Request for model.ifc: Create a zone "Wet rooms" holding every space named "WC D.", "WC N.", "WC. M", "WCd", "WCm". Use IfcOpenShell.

First a look at what the model holds.

```python
import ifcopenshell

model = ifcopenshell.open("model.ifc")
print(model.schema)
seen = {}
for space in model.by_type("IfcSpace"):
    seen[space.LongName] = seen.get(space.LongName, 0) + 1
for name, count in sorted(seen.items(), key=str):
    print(count, "x", name)
print("zones:", [z.Name for z in model.by_type("IfcZone")][:20])
```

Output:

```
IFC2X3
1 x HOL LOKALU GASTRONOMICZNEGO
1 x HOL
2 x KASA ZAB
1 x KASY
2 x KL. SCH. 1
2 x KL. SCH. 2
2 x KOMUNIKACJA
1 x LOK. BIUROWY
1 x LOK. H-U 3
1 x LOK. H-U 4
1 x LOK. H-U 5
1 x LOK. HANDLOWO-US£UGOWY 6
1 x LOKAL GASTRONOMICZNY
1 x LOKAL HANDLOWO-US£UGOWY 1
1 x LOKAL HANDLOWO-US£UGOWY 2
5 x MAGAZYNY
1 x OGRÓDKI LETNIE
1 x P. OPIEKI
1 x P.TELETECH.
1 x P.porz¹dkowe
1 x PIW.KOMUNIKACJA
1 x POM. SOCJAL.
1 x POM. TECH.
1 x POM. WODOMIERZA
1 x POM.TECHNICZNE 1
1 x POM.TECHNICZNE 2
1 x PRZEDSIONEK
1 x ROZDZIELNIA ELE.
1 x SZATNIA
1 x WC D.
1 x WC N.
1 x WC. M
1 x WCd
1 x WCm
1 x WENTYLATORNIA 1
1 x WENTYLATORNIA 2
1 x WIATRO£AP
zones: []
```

```python
import ifcopenshell
import ifcopenshell.api.group
import ifcopenshell.api.root

model = ifcopenshell.open("model.ifc")

names = {"WC D.", "WC N.", "WC. M", "WCd", "WCm"}
spaces = [s for s in model.by_type("IfcSpace") if s.LongName in names]

zone = ifcopenshell.api.root.create_entity(model, ifc_class="IfcZone", name="Wet rooms")
ifcopenshell.api.group.assign_group(model, products=spaces, group=zone)
print(len(spaces), "spaces in", zone.Name)

model.write("model-out.ifc")
```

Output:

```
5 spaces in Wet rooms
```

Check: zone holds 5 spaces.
